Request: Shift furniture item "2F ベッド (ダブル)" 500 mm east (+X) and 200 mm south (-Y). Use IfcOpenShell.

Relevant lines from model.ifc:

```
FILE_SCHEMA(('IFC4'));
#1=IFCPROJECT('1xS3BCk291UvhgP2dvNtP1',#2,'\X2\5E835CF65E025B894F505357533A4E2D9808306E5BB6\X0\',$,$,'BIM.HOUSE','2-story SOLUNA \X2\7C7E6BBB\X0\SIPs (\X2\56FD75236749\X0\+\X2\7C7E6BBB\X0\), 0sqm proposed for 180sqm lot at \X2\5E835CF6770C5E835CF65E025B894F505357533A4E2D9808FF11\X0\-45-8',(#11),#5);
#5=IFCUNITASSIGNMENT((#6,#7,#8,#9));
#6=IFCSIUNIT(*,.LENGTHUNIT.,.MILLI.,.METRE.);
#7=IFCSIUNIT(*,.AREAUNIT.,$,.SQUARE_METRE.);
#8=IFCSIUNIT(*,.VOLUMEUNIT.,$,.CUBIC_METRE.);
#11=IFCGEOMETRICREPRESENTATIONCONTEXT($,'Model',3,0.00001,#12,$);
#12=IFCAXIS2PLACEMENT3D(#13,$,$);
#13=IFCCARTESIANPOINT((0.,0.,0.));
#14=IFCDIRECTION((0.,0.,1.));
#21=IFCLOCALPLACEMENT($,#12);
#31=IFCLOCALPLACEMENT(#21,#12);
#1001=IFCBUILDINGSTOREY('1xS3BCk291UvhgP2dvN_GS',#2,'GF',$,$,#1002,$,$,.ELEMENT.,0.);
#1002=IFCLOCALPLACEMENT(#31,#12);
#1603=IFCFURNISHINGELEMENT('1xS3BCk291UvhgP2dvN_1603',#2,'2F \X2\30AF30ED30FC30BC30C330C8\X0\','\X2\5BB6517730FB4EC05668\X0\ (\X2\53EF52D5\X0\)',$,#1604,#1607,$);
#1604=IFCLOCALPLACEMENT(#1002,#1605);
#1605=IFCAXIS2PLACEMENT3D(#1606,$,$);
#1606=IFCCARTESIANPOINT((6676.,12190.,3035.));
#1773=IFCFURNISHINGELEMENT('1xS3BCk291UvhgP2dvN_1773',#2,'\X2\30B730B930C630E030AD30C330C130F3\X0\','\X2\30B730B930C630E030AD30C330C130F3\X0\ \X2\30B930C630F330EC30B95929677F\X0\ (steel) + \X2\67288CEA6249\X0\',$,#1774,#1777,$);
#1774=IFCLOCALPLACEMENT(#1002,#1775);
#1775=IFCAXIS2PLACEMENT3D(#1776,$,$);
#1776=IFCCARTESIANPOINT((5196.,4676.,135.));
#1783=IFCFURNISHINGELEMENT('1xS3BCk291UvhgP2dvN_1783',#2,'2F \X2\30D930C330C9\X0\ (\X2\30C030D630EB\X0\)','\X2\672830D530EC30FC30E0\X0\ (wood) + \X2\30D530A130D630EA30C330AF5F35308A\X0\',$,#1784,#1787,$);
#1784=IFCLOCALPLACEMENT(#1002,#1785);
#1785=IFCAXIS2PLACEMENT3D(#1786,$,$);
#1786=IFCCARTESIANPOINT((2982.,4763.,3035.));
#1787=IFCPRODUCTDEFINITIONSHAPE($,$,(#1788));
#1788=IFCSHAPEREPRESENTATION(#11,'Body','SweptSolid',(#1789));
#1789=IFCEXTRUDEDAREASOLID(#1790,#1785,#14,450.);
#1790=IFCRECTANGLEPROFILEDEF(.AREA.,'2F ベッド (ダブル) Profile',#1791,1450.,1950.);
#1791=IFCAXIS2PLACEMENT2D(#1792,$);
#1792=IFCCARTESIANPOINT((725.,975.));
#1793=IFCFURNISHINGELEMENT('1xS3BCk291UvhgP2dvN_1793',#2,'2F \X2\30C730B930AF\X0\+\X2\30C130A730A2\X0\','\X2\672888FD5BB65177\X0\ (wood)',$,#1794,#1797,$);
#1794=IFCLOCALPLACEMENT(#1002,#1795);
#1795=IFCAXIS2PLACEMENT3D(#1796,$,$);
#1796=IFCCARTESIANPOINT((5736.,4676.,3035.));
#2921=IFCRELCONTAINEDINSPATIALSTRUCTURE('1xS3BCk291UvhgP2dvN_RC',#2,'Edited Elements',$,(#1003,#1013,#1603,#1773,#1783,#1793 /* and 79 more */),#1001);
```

```python
import ifcopenshell
import ifcopenshell.api.geometry
import ifcopenshell.util.placement
import ifcopenshell.util.unit

model = ifcopenshell.open("model.ifc")
unit_scale = ifcopenshell.util.unit.calculate_unit_scale(model)

item = model.by_guid("1xS3BCk291UvhgP2dvN_1783")
matrix = ifcopenshell.util.placement.get_local_placement(item.ObjectPlacement)
matrix[0, 3] += 0.5 / unit_scale
matrix[1, 3] -= 0.2 / unit_scale
ifcopenshell.api.geometry.edit_object_placement(model, product=item, matrix=matrix, is_si=False)

print(ifcopenshell.util.placement.get_local_placement(item.ObjectPlacement).round(3) + 0.0)

model.write("model-out.ifc")
```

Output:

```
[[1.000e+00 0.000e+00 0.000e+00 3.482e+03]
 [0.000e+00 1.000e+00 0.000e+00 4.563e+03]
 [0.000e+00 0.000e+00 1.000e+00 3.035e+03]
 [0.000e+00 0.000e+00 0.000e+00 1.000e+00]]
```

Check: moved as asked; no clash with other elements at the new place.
